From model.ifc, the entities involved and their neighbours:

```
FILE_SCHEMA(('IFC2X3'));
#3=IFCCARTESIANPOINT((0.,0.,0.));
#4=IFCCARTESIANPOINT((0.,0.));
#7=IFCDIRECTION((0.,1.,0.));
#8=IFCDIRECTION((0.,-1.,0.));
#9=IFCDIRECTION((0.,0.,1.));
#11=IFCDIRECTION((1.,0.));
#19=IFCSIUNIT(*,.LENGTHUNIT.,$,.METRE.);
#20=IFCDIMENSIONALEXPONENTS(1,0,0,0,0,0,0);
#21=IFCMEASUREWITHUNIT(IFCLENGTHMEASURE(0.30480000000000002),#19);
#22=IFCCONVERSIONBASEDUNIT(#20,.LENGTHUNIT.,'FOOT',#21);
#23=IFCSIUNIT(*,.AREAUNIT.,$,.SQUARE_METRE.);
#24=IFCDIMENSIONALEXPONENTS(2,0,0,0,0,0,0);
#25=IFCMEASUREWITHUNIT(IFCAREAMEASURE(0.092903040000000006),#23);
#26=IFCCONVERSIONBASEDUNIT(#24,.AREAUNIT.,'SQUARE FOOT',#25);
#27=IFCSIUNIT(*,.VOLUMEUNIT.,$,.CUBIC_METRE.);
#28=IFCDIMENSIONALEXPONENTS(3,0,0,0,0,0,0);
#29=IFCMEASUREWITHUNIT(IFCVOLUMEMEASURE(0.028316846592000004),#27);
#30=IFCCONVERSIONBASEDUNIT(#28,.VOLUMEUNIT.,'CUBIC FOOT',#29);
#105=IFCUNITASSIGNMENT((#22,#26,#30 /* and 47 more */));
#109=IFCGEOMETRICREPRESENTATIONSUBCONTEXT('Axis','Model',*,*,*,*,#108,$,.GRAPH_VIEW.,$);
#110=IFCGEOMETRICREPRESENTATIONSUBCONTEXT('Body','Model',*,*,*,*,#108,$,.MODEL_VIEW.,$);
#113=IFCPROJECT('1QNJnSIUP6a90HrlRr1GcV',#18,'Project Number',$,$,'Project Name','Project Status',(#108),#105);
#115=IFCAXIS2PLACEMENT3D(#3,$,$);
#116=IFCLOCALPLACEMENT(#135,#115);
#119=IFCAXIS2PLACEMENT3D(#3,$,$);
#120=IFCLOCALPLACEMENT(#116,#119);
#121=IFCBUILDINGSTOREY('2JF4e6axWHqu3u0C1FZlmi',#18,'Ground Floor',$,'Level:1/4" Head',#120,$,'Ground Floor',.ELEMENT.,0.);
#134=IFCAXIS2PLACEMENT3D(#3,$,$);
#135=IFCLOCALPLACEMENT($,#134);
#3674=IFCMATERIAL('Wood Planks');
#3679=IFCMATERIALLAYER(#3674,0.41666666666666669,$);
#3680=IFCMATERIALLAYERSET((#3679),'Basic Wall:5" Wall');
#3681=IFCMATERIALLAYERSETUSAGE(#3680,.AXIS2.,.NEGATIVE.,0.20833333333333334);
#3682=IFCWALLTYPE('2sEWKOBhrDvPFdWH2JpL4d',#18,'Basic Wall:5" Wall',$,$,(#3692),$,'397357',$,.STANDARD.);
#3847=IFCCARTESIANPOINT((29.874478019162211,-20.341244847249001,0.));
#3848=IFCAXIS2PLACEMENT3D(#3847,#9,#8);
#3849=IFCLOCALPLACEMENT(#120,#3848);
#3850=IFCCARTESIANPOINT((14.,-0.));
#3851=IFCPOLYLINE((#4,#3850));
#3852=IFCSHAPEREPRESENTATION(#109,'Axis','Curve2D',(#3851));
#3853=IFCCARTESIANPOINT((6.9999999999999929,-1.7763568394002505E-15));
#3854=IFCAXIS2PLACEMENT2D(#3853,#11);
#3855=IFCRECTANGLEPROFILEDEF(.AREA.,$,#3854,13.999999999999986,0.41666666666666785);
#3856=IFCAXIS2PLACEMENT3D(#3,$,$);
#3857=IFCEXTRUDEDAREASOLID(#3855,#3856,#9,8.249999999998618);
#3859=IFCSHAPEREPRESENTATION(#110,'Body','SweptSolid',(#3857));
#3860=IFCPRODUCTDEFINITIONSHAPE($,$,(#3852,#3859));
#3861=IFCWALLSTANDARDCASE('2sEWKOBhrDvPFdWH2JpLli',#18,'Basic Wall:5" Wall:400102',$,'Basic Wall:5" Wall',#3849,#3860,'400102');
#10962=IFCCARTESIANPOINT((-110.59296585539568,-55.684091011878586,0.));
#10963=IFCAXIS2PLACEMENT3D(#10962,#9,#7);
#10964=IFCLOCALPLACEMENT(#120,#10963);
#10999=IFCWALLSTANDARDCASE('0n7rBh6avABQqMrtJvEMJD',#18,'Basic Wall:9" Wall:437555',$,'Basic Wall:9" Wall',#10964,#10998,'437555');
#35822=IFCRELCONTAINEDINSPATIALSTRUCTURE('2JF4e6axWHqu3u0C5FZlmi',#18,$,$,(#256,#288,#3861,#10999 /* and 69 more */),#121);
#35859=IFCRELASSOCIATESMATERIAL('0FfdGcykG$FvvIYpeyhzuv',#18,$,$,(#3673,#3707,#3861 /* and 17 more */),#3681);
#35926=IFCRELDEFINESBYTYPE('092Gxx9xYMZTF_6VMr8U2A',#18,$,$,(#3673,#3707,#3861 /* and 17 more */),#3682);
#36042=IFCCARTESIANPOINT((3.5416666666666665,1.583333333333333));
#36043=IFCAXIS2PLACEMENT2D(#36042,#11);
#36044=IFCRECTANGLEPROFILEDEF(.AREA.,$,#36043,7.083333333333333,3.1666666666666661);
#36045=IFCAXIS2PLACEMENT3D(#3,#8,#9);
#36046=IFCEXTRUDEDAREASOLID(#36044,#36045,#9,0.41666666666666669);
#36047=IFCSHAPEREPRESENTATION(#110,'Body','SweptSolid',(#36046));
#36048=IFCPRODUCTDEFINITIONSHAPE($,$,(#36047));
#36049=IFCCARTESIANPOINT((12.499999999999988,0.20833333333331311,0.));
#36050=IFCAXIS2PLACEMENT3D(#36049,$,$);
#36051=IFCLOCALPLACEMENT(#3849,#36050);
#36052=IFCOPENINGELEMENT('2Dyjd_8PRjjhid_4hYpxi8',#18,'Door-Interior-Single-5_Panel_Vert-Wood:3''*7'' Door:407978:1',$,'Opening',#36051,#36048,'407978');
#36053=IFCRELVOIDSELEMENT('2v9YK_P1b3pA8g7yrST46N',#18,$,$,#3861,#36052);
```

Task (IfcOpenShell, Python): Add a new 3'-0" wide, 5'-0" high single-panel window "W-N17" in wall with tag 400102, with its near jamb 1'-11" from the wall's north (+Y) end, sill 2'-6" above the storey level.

```python
import numpy as np
import ifcopenshell
import ifcopenshell.api.feature
import ifcopenshell.api.geometry
import ifcopenshell.api.root
import ifcopenshell.api.spatial
import ifcopenshell.api.type
import ifcopenshell.geom
import ifcopenshell.util.element
import ifcopenshell.util.placement
import ifcopenshell.util.representation
import ifcopenshell.util.shape
import ifcopenshell.util.unit

model = ifcopenshell.open("model.ifc")
unit_scale = ifcopenshell.util.unit.calculate_unit_scale(model)
settings = ifcopenshell.geom.settings()


def volume(element):
    """Net volume in cubic metres, openings subtracted."""
    shape = ifcopenshell.geom.create_shape(settings, element)
    return ifcopenshell.util.shape.get_volume(shape.geometry)


wall = model.by_guid("2sEWKOBhrDvPFdWH2JpLli")
storey = ifcopenshell.util.element.get_container(wall, ifc_class="IfcBuildingStorey")
context = ifcopenshell.util.representation.get_context(model, "Model", "Body", "MODEL_VIEW")
before = volume(wall)

width, height, from_end, sill = 0.9144, 1.524, 0.5842, 0.762  # metres

# The wall runs along its own X axis, and the end named is its -X end.
wall_shape = ifcopenshell.geom.create_shape(settings, wall)
x, y, z = ifcopenshell.util.shape.get_vertices(wall_shape.geometry).T
start = x.min() + from_end
face, thickness = float(y.min()), float(y.max() - y.min())
wall_matrix = ifcopenshell.util.placement.get_local_placement(wall.ObjectPlacement)
level = ifcopenshell.util.placement.get_local_placement(storey.ObjectPlacement)[2, 3]


def in_wall(x, y):
    """Placement at x, y metres in the wall's axes, at sill height."""
    matrix = wall_matrix.copy()
    matrix[:, 3] = wall_matrix @ np.array([x / unit_scale, y / unit_scale, 0.0, 1.0])
    matrix[2, 3] = level + sill / unit_scale
    return matrix


# Opening: a box that overshoots both wall faces by 50 mm.
opening = ifcopenshell.api.root.create_entity(model, ifc_class="IfcOpeningElement")
box = ifcopenshell.api.geometry.add_wall_representation(
    model, context=context, length=width, height=height, thickness=thickness + 0.1
)
ifcopenshell.api.geometry.assign_representation(model, product=opening, representation=box)
ifcopenshell.api.geometry.edit_object_placement(model, product=opening, matrix=in_wall(start, face - 0.05), is_si=False)
ifcopenshell.api.feature.add_feature(model, feature=opening, element=wall)

window = ifcopenshell.api.root.create_entity(model, ifc_class="IfcWindow", name="W-N17")
window.OverallWidth, window.OverallHeight = width / unit_scale, height / unit_scale
body = ifcopenshell.api.geometry.add_window_representation(
    model,
    context=context,
    overall_width=window.OverallWidth,
    overall_height=window.OverallHeight,
    partition_type="SINGLE_PANEL",
)
ifcopenshell.api.geometry.assign_representation(model, product=window, representation=body)
ifcopenshell.api.spatial.assign_container(model, products=[window], relating_structure=storey)
fills = ifcopenshell.api.feature.add_filling(model, opening=opening, element=window)
fills.OwnerHistory = window.OwnerHistory  # required in IFC2X3

# IFC2X3 keeps the operation on the window style.
style = ifcopenshell.api.root.create_entity(model, ifc_class="IfcWindowStyle", name="W-N17")
style.OperationType, style.ConstructionType = "SINGLE_PANEL", "NOTDEFINED"
style.ParameterTakesPrecedence = style.Sizeable = False
ifcopenshell.api.type.assign_type(model, related_objects=[window], relating_type=style)

# Centre the window in the wall's thickness.
ifcopenshell.api.geometry.edit_object_placement(model, product=window, matrix=in_wall(start, face), is_si=False)
window_shape = ifcopenshell.geom.create_shape(settings, window)
depth = ifcopenshell.util.shape.get_vertices(window_shape.geometry)[:, 1]
offset = face + thickness / 2 - (depth.min() + depth.max()) / 2
ifcopenshell.api.geometry.edit_object_placement(model, product=window, matrix=in_wall(start, offset), is_si=False)

after = volume(wall)

print(f"wall volume {before:.3f} -> {after:.3f} m3")

model.write("model_rev.ifc")
```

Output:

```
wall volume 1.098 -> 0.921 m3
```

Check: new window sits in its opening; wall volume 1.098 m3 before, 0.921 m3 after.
